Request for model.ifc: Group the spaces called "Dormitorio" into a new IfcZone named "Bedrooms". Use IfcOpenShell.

First a look at what the model holds.

```python
import ifcopenshell

model = ifcopenshell.open("model.ifc")
print(model.schema)
seen = {}
for space in model.by_type("IfcSpace"):
    seen[space.LongName] = seen.get(space.LongName, 0) + 1
for name, count in sorted(seen.items(), key=str):
    print(count, "x", name)
print("zones:", [z.Name for z in model.by_type("IfcZone")][:20])
```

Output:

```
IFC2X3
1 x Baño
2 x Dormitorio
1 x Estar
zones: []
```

```python
import ifcopenshell
import ifcopenshell.api.group
import ifcopenshell.api.root

model = ifcopenshell.open("model.ifc")

names = {"Dormitorio"}
spaces = [s for s in model.by_type("IfcSpace") if s.LongName in names]

zone = ifcopenshell.api.root.create_entity(model, ifc_class="IfcZone", name="Bedrooms")
ifcopenshell.api.group.assign_group(model, products=spaces, group=zone)
print(len(spaces), "spaces in", zone.Name)

model.write("model_edited.ifc")
```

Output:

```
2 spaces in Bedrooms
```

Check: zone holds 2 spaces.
